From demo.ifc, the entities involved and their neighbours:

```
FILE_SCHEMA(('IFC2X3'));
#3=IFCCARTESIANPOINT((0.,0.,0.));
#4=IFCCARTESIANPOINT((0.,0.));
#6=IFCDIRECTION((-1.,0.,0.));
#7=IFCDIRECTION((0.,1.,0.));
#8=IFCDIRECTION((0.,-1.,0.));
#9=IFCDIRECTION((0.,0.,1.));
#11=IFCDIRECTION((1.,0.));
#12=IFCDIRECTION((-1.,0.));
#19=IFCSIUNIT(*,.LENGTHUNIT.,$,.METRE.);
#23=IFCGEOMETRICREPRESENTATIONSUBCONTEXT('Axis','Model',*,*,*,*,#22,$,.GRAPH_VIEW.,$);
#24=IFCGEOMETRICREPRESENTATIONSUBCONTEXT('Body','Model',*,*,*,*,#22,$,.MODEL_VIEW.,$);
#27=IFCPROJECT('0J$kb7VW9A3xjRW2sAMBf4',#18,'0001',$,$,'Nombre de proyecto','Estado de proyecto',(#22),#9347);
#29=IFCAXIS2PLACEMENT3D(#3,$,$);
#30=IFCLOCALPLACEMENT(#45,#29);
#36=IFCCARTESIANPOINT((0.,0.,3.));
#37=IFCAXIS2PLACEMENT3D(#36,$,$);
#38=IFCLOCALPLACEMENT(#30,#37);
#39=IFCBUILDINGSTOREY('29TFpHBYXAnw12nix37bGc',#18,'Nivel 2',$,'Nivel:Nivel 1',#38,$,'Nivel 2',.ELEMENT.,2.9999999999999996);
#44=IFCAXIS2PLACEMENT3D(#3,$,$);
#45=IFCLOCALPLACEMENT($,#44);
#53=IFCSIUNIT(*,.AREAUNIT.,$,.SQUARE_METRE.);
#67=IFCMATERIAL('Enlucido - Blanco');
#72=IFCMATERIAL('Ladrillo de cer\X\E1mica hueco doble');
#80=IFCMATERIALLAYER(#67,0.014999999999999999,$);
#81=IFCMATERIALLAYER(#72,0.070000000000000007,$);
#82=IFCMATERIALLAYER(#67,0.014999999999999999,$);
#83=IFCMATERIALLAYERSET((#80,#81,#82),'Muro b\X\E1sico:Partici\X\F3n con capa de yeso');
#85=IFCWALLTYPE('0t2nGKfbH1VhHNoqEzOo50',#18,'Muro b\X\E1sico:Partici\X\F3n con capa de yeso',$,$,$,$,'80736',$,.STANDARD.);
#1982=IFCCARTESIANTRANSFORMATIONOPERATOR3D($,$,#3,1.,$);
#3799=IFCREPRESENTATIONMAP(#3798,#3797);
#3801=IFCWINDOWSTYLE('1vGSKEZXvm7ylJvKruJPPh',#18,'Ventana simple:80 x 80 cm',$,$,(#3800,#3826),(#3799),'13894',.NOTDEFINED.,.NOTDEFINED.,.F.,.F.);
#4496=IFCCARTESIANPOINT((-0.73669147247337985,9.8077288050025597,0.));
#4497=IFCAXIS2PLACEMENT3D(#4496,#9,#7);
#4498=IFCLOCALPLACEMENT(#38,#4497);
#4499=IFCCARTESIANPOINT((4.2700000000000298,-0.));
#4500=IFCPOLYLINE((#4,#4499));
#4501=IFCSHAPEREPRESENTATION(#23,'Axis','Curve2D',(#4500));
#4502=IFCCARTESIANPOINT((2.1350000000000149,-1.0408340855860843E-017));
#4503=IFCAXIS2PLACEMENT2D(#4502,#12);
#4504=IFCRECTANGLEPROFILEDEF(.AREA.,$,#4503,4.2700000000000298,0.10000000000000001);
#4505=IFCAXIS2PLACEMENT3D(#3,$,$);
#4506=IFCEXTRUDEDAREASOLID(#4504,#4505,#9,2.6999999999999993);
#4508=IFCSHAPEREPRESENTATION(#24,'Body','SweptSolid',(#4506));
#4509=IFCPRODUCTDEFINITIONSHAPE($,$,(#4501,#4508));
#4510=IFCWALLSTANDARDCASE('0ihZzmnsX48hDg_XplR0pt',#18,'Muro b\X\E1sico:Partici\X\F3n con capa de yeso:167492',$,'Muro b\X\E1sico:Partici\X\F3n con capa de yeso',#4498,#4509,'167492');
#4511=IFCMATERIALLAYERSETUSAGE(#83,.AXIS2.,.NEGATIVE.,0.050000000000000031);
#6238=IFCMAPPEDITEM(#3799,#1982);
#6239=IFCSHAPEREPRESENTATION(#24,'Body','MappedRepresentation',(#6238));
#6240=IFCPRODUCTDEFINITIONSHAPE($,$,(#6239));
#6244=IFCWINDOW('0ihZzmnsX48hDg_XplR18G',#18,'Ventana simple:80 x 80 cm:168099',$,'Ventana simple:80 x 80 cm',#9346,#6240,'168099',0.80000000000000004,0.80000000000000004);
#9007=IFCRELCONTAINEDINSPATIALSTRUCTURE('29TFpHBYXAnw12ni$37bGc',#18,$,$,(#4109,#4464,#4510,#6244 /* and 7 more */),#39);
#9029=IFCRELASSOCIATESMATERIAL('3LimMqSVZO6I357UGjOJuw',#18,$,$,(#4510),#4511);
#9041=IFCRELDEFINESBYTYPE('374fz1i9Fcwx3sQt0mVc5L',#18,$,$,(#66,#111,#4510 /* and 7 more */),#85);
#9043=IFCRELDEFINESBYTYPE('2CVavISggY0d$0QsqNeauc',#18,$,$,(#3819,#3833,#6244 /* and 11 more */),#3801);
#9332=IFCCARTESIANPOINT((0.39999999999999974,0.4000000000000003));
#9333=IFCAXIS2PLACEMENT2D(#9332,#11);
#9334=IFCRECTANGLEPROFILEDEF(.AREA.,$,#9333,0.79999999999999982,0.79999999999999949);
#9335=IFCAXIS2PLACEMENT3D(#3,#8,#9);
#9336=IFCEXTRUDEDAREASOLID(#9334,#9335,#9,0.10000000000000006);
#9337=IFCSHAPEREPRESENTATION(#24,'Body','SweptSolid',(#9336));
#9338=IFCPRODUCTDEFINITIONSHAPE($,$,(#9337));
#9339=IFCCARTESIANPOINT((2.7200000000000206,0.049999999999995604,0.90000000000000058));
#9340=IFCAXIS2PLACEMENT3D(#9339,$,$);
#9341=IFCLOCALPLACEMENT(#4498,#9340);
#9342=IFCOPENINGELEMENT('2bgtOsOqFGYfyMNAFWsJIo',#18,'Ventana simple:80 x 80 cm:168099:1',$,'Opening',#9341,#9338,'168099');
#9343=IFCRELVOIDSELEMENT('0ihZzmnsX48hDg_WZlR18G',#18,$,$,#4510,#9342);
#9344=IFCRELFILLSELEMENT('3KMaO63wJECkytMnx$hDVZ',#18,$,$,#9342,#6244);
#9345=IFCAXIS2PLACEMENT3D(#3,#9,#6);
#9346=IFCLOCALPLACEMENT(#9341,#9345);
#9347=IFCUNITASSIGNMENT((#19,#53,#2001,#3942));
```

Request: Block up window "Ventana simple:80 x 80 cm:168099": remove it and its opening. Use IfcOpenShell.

```python
import ifcopenshell
import ifcopenshell.api.feature
import ifcopenshell.api.root
import ifcopenshell.geom
import ifcopenshell.util.shape

model = ifcopenshell.open("demo.ifc")
settings = ifcopenshell.geom.settings()


def volume(element):
    """Net volume in cubic metres, openings subtracted."""
    shape = ifcopenshell.geom.create_shape(settings, element)
    return ifcopenshell.util.shape.get_volume(shape.geometry)


window = model.by_id(6244)
opening = window.FillsVoids[0].RelatingOpeningElement
wall = opening.VoidsElements[0].RelatingBuildingElement
before = volume(wall)

ifcopenshell.api.root.remove_product(model, product=window)
ifcopenshell.api.feature.remove_feature(model, feature=opening)

after = volume(wall)

print(f"wall volume {before:.3f} -> {after:.3f} m3")

model.write("demo-out.ifc")
```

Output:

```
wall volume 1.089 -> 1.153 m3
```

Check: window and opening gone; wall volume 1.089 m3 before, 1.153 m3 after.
